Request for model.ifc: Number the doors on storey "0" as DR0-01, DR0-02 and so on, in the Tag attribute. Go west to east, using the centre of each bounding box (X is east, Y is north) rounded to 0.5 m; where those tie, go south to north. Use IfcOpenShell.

First a look at what the model holds.

```python
import ifcopenshell
import ifcopenshell.util.element
import ifcopenshell.util.placement

model = ifcopenshell.open("model.ifc")
print(model.schema)
storey = next(s for s in model.by_type("IfcBuildingStorey") if s.Name == "0")
doors = [e for e in ifcopenshell.util.element.get_decomposition(storey) if e.is_a("IfcDoor")]
for e in sorted(doors, key=lambda e: e.id()):
    origin = ifcopenshell.util.placement.get_local_placement(e.ObjectPlacement)[:3, 3]
    print(e.id(), e.Tag, e.Name, origin.round(2) + 0.0, sep=" | ")
```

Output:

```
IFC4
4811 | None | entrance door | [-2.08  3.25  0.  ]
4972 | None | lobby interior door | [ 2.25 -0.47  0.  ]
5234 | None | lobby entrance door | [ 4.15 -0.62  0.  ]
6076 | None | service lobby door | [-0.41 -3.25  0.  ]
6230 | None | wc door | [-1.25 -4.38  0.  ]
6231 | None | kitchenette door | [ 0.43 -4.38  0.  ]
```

```python
import ifcopenshell
import ifcopenshell.geom
import ifcopenshell.util.element
import ifcopenshell.util.shape

model = ifcopenshell.open("model.ifc")
settings = ifcopenshell.geom.settings()
settings.set("use-world-coords", True)


def centre(element):
    shape = ifcopenshell.geom.create_shape(settings, element)
    return ifcopenshell.util.shape.get_bbox_centroid(shape.geometry)


storey = next(s for s in model.by_type("IfcBuildingStorey") if s.Name == "0")
doors = [e for e in ifcopenshell.util.element.get_decomposition(storey) if e.is_a("IfcDoor")]

# Insertion points can sit at a corner or the storey origin, so sort by the geometry (in metres).
centres = {e: centre(e) for e in doors}
doors.sort(key=lambda e: (round(centres[e][0] / 0.5), centres[e][1]))

for i, e in enumerate(doors, start=1):
    number = f"DR0-{i:02d}"
    e.Tag = number
    print(e.id(), number)

model.write("model_v2.ifc")
```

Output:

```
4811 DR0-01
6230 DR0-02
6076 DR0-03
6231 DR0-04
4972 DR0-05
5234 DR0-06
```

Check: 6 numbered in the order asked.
